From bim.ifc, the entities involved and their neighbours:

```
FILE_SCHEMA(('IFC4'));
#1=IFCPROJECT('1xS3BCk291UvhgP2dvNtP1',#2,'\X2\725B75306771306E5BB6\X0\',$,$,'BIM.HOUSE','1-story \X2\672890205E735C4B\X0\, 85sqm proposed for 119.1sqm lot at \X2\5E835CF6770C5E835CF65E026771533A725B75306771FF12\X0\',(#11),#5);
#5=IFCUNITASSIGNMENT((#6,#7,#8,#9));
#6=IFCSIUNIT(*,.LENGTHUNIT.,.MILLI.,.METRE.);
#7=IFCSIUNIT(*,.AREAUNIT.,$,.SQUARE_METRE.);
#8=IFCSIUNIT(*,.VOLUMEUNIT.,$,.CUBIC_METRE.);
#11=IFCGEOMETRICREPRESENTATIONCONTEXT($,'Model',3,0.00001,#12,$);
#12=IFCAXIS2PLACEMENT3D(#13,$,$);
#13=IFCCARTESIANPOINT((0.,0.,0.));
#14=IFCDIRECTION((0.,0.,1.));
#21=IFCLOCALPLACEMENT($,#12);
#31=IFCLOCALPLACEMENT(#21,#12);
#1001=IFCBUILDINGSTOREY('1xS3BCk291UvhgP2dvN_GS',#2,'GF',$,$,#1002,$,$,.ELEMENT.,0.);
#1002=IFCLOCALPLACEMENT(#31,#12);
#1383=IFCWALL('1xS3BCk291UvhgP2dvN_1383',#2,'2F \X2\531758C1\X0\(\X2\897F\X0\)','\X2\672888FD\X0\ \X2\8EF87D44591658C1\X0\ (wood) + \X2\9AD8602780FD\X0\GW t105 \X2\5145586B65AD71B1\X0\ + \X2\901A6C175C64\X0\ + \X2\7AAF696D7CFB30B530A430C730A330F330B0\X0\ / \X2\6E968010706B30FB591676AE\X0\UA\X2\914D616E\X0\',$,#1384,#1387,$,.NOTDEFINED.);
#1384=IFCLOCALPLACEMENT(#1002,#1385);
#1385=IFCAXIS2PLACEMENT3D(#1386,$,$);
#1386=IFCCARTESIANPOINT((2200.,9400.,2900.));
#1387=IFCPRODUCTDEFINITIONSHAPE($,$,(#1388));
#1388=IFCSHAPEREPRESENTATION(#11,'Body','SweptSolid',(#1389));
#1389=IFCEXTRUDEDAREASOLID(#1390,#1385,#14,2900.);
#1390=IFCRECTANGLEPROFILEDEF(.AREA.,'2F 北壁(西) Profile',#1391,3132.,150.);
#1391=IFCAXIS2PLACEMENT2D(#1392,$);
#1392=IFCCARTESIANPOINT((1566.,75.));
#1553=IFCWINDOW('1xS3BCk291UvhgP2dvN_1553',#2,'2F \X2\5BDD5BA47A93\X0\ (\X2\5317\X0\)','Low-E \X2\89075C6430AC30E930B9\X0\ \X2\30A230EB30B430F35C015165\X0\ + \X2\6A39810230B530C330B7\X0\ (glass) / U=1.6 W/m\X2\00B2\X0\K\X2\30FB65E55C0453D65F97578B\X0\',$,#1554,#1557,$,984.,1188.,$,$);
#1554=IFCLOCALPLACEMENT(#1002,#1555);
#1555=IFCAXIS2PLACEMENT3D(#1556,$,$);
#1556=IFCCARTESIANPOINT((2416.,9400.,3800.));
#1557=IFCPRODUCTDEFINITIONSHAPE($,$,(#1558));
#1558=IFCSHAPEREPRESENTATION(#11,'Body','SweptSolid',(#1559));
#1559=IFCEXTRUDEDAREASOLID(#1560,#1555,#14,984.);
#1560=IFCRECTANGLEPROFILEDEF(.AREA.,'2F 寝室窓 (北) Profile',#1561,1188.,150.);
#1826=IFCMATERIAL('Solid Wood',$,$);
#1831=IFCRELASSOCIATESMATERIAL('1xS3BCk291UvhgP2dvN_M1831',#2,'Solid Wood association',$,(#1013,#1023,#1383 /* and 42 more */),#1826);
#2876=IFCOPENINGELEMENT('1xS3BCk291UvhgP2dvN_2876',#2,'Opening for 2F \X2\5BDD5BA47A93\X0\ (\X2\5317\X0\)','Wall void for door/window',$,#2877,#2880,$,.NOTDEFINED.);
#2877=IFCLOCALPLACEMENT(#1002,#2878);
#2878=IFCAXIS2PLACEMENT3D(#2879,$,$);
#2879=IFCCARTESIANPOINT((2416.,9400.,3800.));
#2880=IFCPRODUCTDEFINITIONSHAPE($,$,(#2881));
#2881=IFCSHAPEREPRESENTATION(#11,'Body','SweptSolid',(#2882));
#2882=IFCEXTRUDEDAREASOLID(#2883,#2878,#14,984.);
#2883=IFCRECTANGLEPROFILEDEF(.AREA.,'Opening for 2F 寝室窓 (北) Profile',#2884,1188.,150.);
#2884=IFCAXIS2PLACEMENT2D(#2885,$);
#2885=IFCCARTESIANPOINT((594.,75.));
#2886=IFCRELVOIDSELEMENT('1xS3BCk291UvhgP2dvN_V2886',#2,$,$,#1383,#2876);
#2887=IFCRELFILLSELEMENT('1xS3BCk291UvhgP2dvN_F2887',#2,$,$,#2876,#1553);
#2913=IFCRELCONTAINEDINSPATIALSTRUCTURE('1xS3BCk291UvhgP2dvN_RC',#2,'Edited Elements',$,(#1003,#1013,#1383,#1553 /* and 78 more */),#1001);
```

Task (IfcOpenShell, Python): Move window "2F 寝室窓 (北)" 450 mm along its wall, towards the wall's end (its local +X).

```python
import ifcopenshell
import ifcopenshell.api.geometry
import ifcopenshell.util.placement

model = ifcopenshell.open("bim.ifc")

window = model.by_guid("1xS3BCk291UvhgP2dvN_1553")
opening = window.FillsVoids[0].RelatingOpeningElement
wall = opening.VoidsElements[0].RelatingBuildingElement

wall_matrix = ifcopenshell.util.placement.get_local_placement(wall.ObjectPlacement)
shift = wall_matrix[:3, 0] * 450.0
before = ifcopenshell.util.placement.get_local_placement(window.ObjectPlacement)[:3, 3].copy()

# The window is not placed relative to its opening, so move both.
for product in (opening, window):
    matrix = ifcopenshell.util.placement.get_local_placement(product.ObjectPlacement)
    matrix[:3, 3] += shift
    ifcopenshell.api.geometry.edit_object_placement(model, product=product, matrix=matrix, is_si=False)

after = ifcopenshell.util.placement.get_local_placement(window.ObjectPlacement)[:3, 3]
print("window moved by", (after - before).round(3) + 0.0)

model.write("bim_v2.ifc")
```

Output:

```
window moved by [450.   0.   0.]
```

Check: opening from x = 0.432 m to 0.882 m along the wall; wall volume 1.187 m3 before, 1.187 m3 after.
